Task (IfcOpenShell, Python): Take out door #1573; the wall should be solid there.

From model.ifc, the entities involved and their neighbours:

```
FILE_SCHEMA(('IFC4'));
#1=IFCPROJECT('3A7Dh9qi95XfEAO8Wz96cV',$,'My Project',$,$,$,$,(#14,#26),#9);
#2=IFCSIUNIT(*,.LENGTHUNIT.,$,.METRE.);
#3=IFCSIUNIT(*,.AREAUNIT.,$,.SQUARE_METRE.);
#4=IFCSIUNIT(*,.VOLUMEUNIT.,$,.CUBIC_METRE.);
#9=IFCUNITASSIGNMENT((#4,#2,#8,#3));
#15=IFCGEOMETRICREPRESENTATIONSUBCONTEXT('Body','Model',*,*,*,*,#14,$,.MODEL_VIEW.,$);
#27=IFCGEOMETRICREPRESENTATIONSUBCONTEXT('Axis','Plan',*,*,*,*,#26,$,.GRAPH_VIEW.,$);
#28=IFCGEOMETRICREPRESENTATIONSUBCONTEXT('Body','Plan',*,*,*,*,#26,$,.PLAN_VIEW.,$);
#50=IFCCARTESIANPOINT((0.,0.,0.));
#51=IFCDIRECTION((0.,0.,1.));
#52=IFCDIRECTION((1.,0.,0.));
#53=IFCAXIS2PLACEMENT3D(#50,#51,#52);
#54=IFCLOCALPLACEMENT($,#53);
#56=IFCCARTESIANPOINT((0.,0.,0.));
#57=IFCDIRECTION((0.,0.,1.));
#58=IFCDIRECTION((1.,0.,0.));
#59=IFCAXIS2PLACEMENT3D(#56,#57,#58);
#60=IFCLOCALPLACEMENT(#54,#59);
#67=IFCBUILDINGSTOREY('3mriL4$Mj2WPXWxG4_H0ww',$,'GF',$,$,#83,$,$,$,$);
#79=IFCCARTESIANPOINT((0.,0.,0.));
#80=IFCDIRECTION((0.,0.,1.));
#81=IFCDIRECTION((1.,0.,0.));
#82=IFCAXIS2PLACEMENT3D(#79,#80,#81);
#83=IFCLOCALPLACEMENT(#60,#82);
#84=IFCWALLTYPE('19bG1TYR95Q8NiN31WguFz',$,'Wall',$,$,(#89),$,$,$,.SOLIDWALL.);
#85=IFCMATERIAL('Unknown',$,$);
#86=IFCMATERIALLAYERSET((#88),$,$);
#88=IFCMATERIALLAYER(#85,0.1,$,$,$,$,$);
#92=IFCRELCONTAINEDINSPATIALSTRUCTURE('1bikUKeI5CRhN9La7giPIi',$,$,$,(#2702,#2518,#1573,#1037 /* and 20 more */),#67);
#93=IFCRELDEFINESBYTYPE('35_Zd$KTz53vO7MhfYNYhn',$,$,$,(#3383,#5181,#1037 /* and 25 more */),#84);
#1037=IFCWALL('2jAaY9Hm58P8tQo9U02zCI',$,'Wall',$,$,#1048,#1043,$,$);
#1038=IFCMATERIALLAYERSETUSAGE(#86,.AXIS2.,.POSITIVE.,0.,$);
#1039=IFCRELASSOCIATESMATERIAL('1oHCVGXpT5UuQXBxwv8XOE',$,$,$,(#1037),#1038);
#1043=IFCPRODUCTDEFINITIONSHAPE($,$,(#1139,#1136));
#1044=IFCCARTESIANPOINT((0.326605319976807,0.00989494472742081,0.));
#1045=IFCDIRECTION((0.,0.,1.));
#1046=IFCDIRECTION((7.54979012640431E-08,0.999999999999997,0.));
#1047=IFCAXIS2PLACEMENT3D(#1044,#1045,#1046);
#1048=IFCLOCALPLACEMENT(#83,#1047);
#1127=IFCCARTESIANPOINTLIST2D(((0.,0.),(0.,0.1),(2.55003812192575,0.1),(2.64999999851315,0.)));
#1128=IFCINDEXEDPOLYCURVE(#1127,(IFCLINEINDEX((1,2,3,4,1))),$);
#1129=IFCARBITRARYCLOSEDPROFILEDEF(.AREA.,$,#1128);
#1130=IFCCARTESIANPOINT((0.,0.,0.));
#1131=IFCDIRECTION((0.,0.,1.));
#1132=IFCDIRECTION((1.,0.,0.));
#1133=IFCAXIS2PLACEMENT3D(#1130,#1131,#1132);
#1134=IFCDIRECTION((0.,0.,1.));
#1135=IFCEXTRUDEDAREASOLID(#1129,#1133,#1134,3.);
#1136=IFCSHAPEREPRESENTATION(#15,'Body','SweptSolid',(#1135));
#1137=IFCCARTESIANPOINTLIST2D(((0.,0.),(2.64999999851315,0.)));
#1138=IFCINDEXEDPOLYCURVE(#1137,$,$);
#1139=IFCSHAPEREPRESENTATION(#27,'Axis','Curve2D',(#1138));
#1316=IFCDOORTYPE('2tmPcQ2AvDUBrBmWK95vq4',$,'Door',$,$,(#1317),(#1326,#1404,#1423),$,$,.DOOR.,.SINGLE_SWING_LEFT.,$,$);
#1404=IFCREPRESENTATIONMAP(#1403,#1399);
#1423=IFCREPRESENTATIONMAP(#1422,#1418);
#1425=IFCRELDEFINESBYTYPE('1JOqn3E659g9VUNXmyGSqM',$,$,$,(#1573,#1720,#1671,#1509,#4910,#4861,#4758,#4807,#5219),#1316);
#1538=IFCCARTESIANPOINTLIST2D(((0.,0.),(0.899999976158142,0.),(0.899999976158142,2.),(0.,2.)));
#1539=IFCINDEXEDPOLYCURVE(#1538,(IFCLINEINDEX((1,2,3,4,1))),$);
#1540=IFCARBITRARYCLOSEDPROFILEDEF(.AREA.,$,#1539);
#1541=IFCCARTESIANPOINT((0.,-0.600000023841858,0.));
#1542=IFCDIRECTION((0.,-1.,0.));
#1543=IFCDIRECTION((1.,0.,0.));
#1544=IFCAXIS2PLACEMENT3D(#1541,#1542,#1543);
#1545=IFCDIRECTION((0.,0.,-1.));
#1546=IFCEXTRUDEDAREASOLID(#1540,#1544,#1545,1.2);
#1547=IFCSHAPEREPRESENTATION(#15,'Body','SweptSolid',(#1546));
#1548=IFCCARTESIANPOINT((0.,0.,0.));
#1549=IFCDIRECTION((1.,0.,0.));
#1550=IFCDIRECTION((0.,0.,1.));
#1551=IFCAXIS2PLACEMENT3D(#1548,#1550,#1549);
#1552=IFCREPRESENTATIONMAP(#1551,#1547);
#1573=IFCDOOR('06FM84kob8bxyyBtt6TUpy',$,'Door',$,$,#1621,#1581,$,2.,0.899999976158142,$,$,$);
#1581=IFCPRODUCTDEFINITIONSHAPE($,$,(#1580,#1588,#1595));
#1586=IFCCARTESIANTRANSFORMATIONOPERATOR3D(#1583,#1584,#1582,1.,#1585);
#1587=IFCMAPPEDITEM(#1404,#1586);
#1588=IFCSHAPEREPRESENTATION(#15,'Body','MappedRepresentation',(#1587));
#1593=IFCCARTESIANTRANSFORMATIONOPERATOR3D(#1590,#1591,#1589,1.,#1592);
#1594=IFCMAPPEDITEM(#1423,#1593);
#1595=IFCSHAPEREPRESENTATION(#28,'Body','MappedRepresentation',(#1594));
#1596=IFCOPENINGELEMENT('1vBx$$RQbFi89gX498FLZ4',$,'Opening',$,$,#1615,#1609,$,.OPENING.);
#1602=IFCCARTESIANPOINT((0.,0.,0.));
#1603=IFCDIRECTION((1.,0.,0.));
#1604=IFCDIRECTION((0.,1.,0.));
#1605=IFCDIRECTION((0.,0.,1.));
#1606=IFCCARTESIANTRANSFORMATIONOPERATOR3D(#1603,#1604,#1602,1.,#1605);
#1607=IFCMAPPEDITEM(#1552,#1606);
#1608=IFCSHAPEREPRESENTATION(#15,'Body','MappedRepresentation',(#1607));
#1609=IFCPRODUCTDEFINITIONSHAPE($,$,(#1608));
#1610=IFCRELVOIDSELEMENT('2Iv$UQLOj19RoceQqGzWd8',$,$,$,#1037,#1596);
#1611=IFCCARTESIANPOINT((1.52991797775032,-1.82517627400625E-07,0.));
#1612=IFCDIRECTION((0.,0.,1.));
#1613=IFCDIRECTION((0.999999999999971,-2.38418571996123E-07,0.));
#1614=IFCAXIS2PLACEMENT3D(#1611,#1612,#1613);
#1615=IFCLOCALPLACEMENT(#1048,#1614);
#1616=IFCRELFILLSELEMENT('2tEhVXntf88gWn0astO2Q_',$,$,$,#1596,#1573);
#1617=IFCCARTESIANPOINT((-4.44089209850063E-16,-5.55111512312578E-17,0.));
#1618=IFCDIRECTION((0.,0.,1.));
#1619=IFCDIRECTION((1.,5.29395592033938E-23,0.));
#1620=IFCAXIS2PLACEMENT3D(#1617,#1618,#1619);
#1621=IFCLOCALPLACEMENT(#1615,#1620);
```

```python
import ifcopenshell
import ifcopenshell.api.feature
import ifcopenshell.api.root
import ifcopenshell.geom
import ifcopenshell.util.shape

model = ifcopenshell.open("model.ifc")
settings = ifcopenshell.geom.settings()


def volume(element):
    """Net volume in cubic metres, openings subtracted."""
    shape = ifcopenshell.geom.create_shape(settings, element)
    return ifcopenshell.util.shape.get_volume(shape.geometry)


door = model.by_guid("06FM84kob8bxyyBtt6TUpy")
opening = door.FillsVoids[0].RelatingOpeningElement
wall = opening.VoidsElements[0].RelatingBuildingElement
before = volume(wall)

ifcopenshell.api.root.remove_product(model, product=door)
ifcopenshell.api.feature.remove_feature(model, feature=opening)

after = volume(wall)

print(f"wall volume {before:.3f} -> {after:.3f} m3")

model.write("model_v2.ifc")
```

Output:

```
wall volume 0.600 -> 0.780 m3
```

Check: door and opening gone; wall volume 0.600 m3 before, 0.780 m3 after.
